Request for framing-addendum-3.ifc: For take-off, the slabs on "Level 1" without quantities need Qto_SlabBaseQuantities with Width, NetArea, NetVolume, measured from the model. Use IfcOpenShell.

First a look at what the model holds.

```python
import ifcopenshell
import ifcopenshell.util.element
import ifcopenshell.util.unit

model = ifcopenshell.open("framing-addendum-3.ifc")
print(model.schema)
for unit_type in ("LENGTHUNIT", "AREAUNIT", "VOLUMEUNIT"):
    print(unit_type, ifcopenshell.util.unit.calculate_unit_scale(model, unit_type))
storey = next(s for s in model.by_type("IfcBuildingStorey") if s.Name == "Level 1")
slabs = [e for e in ifcopenshell.util.element.get_decomposition(storey) if e.is_a("IfcSlab")]
for e in sorted(slabs, key=lambda e: e.id()):
    print(e.id(), e.is_a(), e.Name, list(ifcopenshell.util.element.get_psets(e, qtos_only=True)), sep=" | ")
```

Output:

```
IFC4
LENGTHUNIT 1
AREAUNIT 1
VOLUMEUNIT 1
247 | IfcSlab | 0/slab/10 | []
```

```python
import ifcopenshell
import ifcopenshell.api.pset
import ifcopenshell.geom
import ifcopenshell.util.element
import ifcopenshell.util.shape
import ifcopenshell.util.unit

model = ifcopenshell.open("framing-addendum-3.ifc")
unit_scale = ifcopenshell.util.unit.calculate_unit_scale(model)
area_scale = ifcopenshell.util.unit.calculate_unit_scale(model, "AREAUNIT")
volume_scale = ifcopenshell.util.unit.calculate_unit_scale(model, "VOLUMEUNIT")
settings = ifcopenshell.geom.settings()

storey = next(s for s in model.by_type("IfcBuildingStorey") if s.Name == "Level 1")
slabs = [e for e in ifcopenshell.util.element.get_decomposition(storey) if e.is_a("IfcSlab")]

for e in sorted(slabs, key=lambda e: e.id()):
    if ifcopenshell.util.element.get_psets(e, qtos_only=True, should_inherit=False):
        continue
    # Geometry comes back in metres, in the element's own axes.
    shape = ifcopenshell.geom.create_shape(settings, e)
    values = {
        "Width": ifcopenshell.util.shape.get_z(shape.geometry) / unit_scale,
        "NetArea": ifcopenshell.util.shape.get_footprint_area(shape.geometry) / area_scale,
        "NetVolume": ifcopenshell.util.shape.get_volume(shape.geometry) / volume_scale,
    }
    qto = ifcopenshell.api.pset.add_qto(model, product=e, name="Qto_SlabBaseQuantities")
    ifcopenshell.api.pset.edit_qto(model, qto=qto, properties=values)
    print(e.id(), {k: round(v, 3) for k, v in values.items()})

model.write("framing-addendum-3_rev.ifc")
```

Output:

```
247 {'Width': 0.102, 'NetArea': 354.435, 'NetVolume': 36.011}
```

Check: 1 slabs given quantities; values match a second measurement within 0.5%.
